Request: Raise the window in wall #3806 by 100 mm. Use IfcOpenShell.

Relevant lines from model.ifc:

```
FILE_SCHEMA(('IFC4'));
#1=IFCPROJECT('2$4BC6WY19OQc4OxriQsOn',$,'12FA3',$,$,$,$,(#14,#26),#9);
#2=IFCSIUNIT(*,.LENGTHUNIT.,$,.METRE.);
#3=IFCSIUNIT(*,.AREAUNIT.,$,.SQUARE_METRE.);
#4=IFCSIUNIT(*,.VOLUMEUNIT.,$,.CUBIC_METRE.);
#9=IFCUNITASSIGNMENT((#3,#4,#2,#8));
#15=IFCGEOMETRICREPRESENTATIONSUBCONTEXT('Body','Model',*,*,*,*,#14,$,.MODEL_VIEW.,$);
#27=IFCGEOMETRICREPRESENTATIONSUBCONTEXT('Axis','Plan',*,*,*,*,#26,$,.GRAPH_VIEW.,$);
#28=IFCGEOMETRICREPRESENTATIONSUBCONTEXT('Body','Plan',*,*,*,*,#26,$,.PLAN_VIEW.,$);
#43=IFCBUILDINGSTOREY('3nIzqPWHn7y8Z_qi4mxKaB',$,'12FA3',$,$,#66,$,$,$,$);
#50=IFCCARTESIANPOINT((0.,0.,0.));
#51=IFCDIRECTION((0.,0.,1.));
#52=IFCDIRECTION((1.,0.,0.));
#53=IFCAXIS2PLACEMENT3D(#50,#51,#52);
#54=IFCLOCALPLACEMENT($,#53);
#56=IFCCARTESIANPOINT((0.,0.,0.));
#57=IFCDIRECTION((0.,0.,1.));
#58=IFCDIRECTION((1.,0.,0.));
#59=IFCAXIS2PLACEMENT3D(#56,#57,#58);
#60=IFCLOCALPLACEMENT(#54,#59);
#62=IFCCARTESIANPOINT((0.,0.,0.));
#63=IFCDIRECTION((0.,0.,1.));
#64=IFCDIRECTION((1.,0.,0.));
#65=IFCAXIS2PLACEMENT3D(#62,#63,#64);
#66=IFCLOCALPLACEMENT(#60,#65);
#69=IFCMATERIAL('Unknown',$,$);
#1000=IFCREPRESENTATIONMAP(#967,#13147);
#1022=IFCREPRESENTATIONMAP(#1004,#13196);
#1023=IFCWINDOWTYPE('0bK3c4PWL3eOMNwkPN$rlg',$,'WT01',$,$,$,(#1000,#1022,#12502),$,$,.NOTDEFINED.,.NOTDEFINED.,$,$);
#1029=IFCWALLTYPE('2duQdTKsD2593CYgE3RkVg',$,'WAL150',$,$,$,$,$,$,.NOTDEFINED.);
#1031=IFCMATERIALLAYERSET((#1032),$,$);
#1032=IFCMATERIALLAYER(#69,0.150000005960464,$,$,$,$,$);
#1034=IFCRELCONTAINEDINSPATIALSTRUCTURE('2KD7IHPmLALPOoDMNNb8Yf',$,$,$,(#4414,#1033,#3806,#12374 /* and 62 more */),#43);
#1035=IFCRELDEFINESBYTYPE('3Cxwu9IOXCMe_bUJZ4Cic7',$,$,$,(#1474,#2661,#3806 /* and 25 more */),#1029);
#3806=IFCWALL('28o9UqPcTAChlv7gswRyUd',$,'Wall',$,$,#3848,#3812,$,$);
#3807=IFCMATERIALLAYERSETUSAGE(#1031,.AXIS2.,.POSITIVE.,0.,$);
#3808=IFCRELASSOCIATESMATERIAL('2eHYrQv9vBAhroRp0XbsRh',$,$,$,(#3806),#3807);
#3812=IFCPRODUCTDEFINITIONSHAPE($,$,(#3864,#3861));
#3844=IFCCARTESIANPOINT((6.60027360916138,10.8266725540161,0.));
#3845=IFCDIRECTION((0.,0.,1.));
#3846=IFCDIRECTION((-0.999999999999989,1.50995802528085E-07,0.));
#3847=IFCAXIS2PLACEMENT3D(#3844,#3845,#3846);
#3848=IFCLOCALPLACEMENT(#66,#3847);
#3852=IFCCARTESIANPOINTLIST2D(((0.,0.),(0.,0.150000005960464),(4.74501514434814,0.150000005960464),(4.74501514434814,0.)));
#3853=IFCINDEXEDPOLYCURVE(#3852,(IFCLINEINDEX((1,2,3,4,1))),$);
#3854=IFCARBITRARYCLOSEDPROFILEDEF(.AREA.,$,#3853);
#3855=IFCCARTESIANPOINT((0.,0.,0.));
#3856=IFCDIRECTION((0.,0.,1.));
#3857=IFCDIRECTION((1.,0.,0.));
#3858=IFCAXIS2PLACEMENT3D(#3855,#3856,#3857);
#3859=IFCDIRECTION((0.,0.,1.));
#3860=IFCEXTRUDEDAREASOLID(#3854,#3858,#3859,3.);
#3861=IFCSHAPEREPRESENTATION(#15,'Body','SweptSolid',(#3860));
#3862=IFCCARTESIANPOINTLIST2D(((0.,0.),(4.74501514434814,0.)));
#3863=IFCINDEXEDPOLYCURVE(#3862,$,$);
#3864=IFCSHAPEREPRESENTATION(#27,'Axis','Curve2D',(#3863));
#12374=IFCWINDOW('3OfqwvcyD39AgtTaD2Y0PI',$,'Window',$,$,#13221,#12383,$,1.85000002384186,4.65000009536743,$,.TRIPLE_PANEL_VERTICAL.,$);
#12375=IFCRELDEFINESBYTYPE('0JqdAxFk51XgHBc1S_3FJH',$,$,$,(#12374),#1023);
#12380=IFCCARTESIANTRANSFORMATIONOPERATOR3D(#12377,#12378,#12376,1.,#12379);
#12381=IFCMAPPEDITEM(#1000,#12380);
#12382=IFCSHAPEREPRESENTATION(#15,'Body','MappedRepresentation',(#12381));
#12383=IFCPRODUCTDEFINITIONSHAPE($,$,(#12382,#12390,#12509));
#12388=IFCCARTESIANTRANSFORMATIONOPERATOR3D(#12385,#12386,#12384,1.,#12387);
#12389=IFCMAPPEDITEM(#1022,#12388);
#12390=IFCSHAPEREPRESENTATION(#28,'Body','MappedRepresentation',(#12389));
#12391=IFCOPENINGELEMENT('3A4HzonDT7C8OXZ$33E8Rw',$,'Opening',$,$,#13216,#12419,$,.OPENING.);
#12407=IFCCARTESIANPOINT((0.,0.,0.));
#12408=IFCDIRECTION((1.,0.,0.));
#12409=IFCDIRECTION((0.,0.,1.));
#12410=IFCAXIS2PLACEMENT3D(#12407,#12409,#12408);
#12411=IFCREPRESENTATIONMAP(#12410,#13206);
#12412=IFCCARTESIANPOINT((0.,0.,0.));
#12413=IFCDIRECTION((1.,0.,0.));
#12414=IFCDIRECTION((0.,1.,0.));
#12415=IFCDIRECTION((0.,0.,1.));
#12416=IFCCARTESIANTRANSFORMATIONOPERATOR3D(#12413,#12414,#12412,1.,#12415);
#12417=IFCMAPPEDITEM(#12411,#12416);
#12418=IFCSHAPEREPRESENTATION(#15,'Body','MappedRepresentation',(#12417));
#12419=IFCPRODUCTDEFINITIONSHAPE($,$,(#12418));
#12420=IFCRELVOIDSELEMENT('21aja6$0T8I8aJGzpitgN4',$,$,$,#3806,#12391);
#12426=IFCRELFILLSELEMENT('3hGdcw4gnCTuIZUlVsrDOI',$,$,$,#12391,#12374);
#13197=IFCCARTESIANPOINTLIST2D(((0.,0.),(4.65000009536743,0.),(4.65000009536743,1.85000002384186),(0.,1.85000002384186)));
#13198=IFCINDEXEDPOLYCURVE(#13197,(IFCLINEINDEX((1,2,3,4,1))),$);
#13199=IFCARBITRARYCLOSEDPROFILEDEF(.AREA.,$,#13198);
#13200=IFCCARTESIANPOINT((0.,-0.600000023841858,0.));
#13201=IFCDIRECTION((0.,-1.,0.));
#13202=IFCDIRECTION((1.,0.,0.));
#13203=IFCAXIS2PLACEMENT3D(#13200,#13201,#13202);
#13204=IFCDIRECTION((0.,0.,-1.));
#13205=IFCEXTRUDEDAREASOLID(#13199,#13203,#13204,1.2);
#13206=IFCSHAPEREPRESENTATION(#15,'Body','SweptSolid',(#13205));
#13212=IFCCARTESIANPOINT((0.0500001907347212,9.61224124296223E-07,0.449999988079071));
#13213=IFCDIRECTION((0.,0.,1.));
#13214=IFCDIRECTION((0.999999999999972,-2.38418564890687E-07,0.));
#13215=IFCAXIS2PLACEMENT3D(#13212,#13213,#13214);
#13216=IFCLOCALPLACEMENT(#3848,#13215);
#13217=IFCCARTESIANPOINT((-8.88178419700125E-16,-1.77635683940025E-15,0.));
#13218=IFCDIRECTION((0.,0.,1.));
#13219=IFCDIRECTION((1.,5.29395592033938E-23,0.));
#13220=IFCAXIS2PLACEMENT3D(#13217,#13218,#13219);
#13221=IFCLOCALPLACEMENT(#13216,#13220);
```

```python
import numpy as np
import ifcopenshell
import ifcopenshell.api.geometry
import ifcopenshell.util.placement
import ifcopenshell.util.unit

model = ifcopenshell.open("model.ifc")
unit_scale = ifcopenshell.util.unit.calculate_unit_scale(model)

window = model.by_id(12374)
opening = window.FillsVoids[0].RelatingOpeningElement
dz = 0.1 / unit_scale

shift = np.array([0.0, 0.0, dz])
# The window is placed relative to its opening, so it follows when the opening moves.
matrix = ifcopenshell.util.placement.get_local_placement(opening.ObjectPlacement)
matrix[:3, 3] += shift
ifcopenshell.api.geometry.edit_object_placement(
    model, product=opening, matrix=matrix, is_si=False, should_transform_children=True
)

print(f"moved by {dz * unit_scale:+.3f} m")

model.write("model_edited.ifc")
```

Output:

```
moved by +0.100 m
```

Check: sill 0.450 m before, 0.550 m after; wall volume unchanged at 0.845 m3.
